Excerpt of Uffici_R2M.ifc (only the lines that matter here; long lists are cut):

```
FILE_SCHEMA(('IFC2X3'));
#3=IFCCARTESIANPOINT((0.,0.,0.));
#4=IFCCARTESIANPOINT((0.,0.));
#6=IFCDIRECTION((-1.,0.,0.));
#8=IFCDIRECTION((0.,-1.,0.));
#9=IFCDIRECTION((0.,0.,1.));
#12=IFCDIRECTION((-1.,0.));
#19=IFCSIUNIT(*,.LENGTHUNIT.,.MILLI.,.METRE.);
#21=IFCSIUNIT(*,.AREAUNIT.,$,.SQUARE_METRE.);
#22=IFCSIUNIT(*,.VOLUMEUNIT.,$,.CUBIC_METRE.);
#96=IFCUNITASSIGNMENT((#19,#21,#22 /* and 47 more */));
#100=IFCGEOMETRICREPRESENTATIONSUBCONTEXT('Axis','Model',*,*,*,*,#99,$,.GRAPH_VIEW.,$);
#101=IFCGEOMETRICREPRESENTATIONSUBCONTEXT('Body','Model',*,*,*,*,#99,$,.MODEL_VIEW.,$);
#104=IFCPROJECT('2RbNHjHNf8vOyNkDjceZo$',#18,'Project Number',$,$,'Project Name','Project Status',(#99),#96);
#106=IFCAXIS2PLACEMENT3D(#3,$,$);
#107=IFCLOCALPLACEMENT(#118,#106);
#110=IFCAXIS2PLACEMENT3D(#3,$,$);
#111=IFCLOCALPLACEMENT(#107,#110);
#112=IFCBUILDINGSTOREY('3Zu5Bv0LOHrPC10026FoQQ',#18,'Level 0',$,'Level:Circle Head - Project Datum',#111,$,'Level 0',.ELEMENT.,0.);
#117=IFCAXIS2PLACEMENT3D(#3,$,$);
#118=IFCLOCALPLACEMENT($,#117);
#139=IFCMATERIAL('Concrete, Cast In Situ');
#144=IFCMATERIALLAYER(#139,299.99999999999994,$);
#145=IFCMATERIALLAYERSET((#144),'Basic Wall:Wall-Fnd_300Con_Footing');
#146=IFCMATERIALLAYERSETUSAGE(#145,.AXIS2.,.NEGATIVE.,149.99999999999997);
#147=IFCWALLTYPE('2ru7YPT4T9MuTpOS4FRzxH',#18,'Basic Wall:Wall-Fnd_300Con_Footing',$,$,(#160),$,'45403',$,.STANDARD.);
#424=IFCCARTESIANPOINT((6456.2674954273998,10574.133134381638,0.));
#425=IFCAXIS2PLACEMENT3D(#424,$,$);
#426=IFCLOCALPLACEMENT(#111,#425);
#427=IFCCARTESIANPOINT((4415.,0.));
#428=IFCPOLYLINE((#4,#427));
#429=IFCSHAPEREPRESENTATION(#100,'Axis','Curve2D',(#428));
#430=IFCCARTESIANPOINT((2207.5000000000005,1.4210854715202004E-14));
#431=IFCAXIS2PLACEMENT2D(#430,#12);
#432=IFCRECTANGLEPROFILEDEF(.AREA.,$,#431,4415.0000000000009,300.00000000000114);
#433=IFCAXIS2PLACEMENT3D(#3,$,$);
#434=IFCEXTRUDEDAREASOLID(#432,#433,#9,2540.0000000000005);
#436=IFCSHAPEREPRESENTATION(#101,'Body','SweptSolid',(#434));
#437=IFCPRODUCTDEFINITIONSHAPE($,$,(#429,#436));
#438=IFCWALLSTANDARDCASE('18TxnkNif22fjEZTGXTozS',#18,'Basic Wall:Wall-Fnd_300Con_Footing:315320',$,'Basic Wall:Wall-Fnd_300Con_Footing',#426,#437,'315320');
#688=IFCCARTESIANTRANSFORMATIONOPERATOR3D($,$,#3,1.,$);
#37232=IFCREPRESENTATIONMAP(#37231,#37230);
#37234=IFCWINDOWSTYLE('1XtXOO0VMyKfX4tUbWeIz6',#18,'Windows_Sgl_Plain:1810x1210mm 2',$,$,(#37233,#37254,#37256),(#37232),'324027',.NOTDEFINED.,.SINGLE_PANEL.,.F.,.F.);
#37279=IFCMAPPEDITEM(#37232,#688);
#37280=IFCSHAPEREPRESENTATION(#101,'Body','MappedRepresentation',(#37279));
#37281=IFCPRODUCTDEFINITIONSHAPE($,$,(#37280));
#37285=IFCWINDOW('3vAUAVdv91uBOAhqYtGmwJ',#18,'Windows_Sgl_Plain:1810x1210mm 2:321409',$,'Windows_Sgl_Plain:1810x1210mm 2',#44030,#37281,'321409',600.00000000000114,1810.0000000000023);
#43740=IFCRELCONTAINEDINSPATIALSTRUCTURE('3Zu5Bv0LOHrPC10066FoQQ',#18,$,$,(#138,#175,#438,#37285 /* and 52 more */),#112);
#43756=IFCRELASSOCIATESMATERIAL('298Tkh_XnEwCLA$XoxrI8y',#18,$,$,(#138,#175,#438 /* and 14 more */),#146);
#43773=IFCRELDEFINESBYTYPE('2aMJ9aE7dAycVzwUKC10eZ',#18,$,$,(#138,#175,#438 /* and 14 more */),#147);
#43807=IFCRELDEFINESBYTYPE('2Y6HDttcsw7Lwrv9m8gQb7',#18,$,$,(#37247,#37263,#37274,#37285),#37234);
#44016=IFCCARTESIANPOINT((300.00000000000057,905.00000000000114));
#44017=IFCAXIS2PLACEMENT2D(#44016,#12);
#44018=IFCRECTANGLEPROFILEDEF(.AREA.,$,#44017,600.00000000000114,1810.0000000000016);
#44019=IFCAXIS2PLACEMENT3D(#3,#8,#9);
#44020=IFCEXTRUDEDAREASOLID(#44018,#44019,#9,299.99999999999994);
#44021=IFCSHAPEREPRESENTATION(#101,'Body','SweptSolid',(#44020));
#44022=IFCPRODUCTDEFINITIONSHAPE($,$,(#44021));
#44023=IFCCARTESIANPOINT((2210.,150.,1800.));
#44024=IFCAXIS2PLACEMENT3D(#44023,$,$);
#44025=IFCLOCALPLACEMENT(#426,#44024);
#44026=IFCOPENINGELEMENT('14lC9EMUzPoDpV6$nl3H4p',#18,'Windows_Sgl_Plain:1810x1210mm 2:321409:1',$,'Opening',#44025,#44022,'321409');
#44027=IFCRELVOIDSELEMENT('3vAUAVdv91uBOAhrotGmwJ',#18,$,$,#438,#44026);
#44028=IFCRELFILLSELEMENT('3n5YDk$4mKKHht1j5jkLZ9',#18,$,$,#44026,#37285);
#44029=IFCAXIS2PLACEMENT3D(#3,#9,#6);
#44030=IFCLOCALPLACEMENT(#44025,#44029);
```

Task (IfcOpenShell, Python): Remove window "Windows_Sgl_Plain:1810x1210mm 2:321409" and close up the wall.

```python
import ifcopenshell
import ifcopenshell.api.feature
import ifcopenshell.api.root
import ifcopenshell.geom
import ifcopenshell.util.shape

model = ifcopenshell.open("Uffici_R2M.ifc")
settings = ifcopenshell.geom.settings()


def volume(element):
    """Net volume in cubic metres, openings subtracted."""
    shape = ifcopenshell.geom.create_shape(settings, element)
    return ifcopenshell.util.shape.get_volume(shape.geometry)


window = model.by_guid("3vAUAVdv91uBOAhqYtGmwJ")
opening = window.FillsVoids[0].RelatingOpeningElement
wall = opening.VoidsElements[0].RelatingBuildingElement
before = volume(wall)

ifcopenshell.api.root.remove_product(model, product=window)
ifcopenshell.api.feature.remove_feature(model, feature=opening)

after = volume(wall)

print(f"wall volume {before:.3f} -> {after:.3f} m3")

model.write("Uffici_R2M_updated.ifc")
```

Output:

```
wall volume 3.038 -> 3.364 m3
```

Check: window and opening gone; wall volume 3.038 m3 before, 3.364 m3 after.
